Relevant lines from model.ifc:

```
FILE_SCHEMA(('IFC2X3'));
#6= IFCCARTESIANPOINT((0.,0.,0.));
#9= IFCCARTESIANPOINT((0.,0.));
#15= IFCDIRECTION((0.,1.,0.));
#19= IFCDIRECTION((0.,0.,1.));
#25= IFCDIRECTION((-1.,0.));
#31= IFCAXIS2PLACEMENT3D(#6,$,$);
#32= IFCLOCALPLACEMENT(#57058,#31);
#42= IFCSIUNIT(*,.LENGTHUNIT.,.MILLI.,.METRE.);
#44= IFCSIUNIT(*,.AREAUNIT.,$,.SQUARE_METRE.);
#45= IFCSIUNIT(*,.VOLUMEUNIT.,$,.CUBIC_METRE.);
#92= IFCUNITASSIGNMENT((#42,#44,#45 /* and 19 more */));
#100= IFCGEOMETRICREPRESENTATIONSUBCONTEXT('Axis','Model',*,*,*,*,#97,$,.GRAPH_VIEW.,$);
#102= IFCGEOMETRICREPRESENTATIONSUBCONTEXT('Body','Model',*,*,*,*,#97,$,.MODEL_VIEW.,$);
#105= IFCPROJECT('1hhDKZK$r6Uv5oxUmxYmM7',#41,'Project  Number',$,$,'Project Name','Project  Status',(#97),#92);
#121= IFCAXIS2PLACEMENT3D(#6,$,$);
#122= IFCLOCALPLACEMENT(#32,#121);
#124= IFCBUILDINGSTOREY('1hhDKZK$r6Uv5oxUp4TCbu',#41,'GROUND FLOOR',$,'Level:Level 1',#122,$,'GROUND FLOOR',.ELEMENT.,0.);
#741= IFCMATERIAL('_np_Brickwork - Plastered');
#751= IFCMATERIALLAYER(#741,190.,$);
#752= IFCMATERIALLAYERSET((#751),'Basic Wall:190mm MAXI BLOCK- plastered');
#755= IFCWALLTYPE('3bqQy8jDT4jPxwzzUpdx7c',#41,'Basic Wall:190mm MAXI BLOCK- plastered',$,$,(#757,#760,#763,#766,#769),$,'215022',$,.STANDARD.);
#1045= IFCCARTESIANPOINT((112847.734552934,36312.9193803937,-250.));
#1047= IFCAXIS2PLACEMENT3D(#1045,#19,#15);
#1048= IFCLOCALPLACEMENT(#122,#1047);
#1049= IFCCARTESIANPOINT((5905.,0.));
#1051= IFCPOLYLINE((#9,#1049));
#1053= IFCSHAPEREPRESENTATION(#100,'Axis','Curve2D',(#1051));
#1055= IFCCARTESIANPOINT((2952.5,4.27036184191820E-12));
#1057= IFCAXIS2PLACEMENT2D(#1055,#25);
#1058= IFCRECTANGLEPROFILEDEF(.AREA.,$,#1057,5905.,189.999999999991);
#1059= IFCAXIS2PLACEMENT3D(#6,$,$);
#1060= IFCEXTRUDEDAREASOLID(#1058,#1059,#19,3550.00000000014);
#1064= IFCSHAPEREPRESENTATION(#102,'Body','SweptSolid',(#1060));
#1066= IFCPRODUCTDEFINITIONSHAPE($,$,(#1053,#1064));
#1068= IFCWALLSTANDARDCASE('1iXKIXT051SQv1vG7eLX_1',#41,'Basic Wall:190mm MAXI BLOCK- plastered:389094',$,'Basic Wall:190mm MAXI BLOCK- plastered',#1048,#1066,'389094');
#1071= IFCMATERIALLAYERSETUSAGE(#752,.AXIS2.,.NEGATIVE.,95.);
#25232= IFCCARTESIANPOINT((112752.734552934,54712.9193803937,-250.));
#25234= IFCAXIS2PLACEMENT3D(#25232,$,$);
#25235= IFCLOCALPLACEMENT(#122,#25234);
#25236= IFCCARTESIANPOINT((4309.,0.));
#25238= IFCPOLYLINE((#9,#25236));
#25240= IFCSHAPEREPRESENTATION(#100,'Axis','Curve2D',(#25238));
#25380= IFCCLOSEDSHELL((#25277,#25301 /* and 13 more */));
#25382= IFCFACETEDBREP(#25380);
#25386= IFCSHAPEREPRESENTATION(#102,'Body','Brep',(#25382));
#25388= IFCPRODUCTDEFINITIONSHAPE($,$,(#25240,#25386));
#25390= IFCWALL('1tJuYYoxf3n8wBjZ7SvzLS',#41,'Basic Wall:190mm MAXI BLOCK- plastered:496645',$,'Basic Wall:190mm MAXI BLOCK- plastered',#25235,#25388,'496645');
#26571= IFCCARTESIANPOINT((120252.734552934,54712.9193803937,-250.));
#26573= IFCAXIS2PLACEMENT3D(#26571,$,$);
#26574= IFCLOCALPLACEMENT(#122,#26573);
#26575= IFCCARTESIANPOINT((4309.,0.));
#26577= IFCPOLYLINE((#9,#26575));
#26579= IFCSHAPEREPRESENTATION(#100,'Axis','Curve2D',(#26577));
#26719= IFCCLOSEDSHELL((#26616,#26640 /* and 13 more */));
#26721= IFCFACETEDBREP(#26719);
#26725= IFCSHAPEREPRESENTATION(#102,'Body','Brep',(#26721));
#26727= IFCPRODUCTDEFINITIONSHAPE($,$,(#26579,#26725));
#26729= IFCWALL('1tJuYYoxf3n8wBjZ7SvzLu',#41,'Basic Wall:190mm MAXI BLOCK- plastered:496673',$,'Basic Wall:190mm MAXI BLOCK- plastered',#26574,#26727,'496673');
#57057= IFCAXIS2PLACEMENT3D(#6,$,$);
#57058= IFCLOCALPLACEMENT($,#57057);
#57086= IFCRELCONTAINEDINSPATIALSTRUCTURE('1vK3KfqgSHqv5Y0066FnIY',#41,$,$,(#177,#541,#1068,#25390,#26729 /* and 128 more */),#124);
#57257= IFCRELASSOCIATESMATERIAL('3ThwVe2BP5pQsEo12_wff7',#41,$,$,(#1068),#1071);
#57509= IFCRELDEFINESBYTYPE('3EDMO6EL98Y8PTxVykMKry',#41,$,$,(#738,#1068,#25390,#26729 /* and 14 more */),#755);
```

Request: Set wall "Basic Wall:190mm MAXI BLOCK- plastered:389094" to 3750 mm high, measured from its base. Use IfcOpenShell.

```python
import ifcopenshell
import ifcopenshell.geom
import ifcopenshell.util.representation
import ifcopenshell.util.shape
import ifcopenshell.util.unit

model = ifcopenshell.open("model.ifc")
unit_scale = ifcopenshell.util.unit.calculate_unit_scale(model)
settings = ifcopenshell.geom.settings()


def volume(element):
    """Net volume in cubic metres, openings subtracted."""
    shape = ifcopenshell.geom.create_shape(settings, element)
    return ifcopenshell.util.shape.get_volume(shape.geometry)


wall = model.by_guid("1iXKIXT051SQv1vG7eLX_1")
before = volume(wall)

body = ifcopenshell.util.representation.get_representation(wall, "Model", "Body")
solid = body.Items[0]
old_height = solid.Depth
solid.Depth = 3.75 / unit_scale
after = volume(wall)

print(f"height {old_height:g} -> {solid.Depth:g}, volume {before:.3f} -> {after:.3f} m3")

model.write("model_updated.ifc")
```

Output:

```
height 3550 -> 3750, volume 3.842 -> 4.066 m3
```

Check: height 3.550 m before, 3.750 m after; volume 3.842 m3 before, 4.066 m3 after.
